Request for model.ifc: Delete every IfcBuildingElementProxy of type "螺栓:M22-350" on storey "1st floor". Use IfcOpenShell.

First a look at what the model holds.

```python
import ifcopenshell
import ifcopenshell.util.element

model = ifcopenshell.open("model.ifc")
print(model.schema)
storey = next(s for s in model.by_type("IfcBuildingStorey") if s.Name == "1st floor")
proxies = [e for e in ifcopenshell.util.element.get_decomposition(storey) if e.is_a("IfcBuildingElementProxy")]
seen = {}
for e in proxies:
    element_type = ifcopenshell.util.element.get_type(e)
    name = element_type.Name if element_type not in (None, e) else None
    seen[name] = seen.get(name, 0) + 1
for name, count in sorted(seen.items(), key=str):
    print(count, "x", name)
```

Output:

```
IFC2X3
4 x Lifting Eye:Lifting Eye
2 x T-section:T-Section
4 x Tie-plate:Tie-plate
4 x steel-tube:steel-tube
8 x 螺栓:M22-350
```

```python
import ifcopenshell
import ifcopenshell.api.root
import ifcopenshell.util.element

model = ifcopenshell.open("model.ifc")

storey = next(s for s in model.by_type("IfcBuildingStorey") if s.Name == "1st floor")
proxies = [e for e in ifcopenshell.util.element.get_decomposition(storey) if e.is_a("IfcBuildingElementProxy")]
targets = [e for e in proxies if (t := ifcopenshell.util.element.get_type(e)) not in (None, e) and t.Name == "螺栓:M22-350"]

for e in targets:
    ifcopenshell.api.root.remove_product(model, product=e)
print(len(targets), "removed")

model.write("model_rev.ifc")
```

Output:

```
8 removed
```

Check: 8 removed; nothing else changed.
